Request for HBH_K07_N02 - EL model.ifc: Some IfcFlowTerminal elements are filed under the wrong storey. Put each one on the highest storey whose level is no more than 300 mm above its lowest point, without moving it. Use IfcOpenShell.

First a look at what the model holds.

```python
import ifcopenshell
import ifcopenshell.util.element
import ifcopenshell.util.placement

model = ifcopenshell.open("HBH_K07_N02 - EL model.ifc")
print(model.schema)
for storey in model.by_type("IfcBuildingStorey"):
    level = ifcopenshell.util.placement.get_storey_elevation(storey)
    count = sum(e.is_a("IfcFlowTerminal") for e in ifcopenshell.util.element.get_contained(storey))
    print(storey.id(), storey.Name, round(level, 3), count, sep=" | ")
```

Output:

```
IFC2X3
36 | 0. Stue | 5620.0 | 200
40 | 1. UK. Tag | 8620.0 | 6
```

```python
import ifcopenshell
import ifcopenshell.api.spatial
import ifcopenshell.geom
import ifcopenshell.util.element
import ifcopenshell.util.placement
import ifcopenshell.util.shape
import ifcopenshell.util.unit

model = ifcopenshell.open("HBH_K07_N02 - EL model.ifc")
unit_scale = ifcopenshell.util.unit.calculate_unit_scale(model)
settings = ifcopenshell.geom.settings()

levels = sorted(
    ((ifcopenshell.util.placement.get_storey_elevation(s) * unit_scale, s) for s in model.by_type("IfcBuildingStorey")),
    key=lambda pair: pair[0],
)

for e in model.by_type("IfcFlowTerminal"):
    current = e.ContainedInStructure[0].RelatingStructure if e.ContainedInStructure else None
    if current is None or not current.is_a("IfcBuildingStorey"):
        continue
    shape = ifcopenshell.geom.create_shape(settings, e)
    bottom = ifcopenshell.util.shape.get_shape_bottom_elevation(shape, shape.geometry)
    below = [s for level, s in levels if level <= bottom + 0.3]
    storey = below[-1] if below else levels[0][1]
    if storey != current:
        # assign_container keeps the world position.
        ifcopenshell.api.spatial.assign_container(model, products=[e], relating_structure=storey)
        print(e.id(), current.Name, "->", storey.Name)

model.write("HBH_K07_N02 - EL model_rev.ifc")
```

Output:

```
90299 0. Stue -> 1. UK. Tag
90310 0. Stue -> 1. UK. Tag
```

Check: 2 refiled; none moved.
